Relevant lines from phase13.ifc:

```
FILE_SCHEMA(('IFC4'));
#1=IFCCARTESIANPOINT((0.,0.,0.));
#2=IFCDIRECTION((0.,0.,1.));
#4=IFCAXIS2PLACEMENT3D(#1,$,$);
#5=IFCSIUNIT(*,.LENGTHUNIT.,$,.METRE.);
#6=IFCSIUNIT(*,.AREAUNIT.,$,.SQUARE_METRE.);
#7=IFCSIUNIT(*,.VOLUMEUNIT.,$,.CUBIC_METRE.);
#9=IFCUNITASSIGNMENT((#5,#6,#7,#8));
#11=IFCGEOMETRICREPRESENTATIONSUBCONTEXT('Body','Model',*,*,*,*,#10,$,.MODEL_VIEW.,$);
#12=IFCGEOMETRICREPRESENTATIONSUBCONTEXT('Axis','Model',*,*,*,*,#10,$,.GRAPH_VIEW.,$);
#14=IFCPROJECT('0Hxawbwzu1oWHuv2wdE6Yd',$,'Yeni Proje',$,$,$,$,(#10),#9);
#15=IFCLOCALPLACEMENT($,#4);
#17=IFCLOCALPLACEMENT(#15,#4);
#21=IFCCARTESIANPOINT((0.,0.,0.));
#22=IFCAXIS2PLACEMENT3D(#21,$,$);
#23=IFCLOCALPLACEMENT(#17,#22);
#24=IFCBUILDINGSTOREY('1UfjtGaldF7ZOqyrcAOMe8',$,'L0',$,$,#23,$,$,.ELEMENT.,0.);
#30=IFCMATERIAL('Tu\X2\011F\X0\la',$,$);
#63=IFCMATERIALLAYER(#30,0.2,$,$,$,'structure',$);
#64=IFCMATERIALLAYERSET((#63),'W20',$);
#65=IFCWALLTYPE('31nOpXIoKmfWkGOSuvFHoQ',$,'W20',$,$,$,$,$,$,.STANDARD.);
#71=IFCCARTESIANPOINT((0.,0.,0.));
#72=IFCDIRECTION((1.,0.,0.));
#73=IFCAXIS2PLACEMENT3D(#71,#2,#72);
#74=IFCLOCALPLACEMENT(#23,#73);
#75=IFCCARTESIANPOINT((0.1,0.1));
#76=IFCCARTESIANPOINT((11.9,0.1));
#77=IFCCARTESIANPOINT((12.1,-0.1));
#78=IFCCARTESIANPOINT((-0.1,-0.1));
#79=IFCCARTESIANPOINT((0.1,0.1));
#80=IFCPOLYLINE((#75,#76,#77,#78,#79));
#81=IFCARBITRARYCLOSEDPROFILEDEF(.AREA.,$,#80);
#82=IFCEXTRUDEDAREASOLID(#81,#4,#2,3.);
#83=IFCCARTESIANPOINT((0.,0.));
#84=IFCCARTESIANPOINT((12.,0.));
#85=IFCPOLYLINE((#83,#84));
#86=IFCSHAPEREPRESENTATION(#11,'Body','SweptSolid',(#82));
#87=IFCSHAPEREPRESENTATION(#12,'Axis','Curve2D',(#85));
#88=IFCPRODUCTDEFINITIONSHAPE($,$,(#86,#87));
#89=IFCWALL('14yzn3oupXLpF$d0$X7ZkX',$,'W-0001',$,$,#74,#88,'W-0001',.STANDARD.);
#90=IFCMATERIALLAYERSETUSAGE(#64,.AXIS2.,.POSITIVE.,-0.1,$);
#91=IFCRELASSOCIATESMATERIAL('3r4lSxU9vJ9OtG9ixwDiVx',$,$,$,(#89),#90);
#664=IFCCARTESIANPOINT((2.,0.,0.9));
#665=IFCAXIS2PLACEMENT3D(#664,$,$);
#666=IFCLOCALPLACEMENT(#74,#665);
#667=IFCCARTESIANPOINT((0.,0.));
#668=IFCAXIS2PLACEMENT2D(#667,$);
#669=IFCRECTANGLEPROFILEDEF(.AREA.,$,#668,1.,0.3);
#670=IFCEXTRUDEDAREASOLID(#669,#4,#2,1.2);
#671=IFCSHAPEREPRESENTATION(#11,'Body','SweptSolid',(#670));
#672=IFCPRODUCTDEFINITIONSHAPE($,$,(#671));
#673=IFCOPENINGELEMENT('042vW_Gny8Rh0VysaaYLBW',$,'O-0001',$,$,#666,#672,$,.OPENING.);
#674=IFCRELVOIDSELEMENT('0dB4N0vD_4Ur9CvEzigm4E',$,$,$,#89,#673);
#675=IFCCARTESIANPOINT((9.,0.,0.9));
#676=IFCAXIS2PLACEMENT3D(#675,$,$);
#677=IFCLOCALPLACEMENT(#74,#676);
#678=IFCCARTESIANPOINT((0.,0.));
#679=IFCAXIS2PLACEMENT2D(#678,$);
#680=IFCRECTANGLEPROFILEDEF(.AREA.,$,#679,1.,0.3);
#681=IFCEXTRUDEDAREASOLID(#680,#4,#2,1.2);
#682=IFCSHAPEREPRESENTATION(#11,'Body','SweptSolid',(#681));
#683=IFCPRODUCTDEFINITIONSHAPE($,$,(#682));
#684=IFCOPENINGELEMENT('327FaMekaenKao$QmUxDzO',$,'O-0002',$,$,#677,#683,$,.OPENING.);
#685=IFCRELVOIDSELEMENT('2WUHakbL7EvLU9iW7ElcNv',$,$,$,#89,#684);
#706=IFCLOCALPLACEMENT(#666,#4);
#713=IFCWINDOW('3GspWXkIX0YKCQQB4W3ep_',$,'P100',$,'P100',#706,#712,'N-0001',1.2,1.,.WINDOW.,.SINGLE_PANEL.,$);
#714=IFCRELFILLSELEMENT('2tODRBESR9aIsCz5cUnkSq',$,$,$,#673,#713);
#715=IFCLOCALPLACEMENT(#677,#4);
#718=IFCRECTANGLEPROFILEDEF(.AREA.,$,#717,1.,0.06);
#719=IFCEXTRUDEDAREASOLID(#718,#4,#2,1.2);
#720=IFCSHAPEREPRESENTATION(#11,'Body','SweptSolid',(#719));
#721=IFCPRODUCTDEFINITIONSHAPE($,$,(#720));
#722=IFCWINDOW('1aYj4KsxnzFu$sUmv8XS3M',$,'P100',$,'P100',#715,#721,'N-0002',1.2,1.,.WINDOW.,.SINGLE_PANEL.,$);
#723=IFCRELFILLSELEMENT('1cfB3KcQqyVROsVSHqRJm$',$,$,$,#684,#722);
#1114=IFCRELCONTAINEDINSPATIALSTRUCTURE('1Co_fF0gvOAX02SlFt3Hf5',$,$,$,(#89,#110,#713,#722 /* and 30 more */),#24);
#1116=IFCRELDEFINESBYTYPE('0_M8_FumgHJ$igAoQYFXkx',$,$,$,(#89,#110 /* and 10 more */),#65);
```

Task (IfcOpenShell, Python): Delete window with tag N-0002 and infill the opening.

```python
import ifcopenshell
import ifcopenshell.api.feature
import ifcopenshell.api.root
import ifcopenshell.geom
import ifcopenshell.util.shape

model = ifcopenshell.open("phase13.ifc")
settings = ifcopenshell.geom.settings()


def volume(element):
    """Net volume in cubic metres, openings subtracted."""
    shape = ifcopenshell.geom.create_shape(settings, element)
    return ifcopenshell.util.shape.get_volume(shape.geometry)


window = model.by_id(722)
opening = window.FillsVoids[0].RelatingOpeningElement
wall = opening.VoidsElements[0].RelatingBuildingElement
before = volume(wall)

ifcopenshell.api.root.remove_product(model, product=window)
ifcopenshell.api.feature.remove_feature(model, feature=opening)

after = volume(wall)

print(f"wall volume {before:.3f} -> {after:.3f} m3")

model.write("phase13_rev.ifc")
```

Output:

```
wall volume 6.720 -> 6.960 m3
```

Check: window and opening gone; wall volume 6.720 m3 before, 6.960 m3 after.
